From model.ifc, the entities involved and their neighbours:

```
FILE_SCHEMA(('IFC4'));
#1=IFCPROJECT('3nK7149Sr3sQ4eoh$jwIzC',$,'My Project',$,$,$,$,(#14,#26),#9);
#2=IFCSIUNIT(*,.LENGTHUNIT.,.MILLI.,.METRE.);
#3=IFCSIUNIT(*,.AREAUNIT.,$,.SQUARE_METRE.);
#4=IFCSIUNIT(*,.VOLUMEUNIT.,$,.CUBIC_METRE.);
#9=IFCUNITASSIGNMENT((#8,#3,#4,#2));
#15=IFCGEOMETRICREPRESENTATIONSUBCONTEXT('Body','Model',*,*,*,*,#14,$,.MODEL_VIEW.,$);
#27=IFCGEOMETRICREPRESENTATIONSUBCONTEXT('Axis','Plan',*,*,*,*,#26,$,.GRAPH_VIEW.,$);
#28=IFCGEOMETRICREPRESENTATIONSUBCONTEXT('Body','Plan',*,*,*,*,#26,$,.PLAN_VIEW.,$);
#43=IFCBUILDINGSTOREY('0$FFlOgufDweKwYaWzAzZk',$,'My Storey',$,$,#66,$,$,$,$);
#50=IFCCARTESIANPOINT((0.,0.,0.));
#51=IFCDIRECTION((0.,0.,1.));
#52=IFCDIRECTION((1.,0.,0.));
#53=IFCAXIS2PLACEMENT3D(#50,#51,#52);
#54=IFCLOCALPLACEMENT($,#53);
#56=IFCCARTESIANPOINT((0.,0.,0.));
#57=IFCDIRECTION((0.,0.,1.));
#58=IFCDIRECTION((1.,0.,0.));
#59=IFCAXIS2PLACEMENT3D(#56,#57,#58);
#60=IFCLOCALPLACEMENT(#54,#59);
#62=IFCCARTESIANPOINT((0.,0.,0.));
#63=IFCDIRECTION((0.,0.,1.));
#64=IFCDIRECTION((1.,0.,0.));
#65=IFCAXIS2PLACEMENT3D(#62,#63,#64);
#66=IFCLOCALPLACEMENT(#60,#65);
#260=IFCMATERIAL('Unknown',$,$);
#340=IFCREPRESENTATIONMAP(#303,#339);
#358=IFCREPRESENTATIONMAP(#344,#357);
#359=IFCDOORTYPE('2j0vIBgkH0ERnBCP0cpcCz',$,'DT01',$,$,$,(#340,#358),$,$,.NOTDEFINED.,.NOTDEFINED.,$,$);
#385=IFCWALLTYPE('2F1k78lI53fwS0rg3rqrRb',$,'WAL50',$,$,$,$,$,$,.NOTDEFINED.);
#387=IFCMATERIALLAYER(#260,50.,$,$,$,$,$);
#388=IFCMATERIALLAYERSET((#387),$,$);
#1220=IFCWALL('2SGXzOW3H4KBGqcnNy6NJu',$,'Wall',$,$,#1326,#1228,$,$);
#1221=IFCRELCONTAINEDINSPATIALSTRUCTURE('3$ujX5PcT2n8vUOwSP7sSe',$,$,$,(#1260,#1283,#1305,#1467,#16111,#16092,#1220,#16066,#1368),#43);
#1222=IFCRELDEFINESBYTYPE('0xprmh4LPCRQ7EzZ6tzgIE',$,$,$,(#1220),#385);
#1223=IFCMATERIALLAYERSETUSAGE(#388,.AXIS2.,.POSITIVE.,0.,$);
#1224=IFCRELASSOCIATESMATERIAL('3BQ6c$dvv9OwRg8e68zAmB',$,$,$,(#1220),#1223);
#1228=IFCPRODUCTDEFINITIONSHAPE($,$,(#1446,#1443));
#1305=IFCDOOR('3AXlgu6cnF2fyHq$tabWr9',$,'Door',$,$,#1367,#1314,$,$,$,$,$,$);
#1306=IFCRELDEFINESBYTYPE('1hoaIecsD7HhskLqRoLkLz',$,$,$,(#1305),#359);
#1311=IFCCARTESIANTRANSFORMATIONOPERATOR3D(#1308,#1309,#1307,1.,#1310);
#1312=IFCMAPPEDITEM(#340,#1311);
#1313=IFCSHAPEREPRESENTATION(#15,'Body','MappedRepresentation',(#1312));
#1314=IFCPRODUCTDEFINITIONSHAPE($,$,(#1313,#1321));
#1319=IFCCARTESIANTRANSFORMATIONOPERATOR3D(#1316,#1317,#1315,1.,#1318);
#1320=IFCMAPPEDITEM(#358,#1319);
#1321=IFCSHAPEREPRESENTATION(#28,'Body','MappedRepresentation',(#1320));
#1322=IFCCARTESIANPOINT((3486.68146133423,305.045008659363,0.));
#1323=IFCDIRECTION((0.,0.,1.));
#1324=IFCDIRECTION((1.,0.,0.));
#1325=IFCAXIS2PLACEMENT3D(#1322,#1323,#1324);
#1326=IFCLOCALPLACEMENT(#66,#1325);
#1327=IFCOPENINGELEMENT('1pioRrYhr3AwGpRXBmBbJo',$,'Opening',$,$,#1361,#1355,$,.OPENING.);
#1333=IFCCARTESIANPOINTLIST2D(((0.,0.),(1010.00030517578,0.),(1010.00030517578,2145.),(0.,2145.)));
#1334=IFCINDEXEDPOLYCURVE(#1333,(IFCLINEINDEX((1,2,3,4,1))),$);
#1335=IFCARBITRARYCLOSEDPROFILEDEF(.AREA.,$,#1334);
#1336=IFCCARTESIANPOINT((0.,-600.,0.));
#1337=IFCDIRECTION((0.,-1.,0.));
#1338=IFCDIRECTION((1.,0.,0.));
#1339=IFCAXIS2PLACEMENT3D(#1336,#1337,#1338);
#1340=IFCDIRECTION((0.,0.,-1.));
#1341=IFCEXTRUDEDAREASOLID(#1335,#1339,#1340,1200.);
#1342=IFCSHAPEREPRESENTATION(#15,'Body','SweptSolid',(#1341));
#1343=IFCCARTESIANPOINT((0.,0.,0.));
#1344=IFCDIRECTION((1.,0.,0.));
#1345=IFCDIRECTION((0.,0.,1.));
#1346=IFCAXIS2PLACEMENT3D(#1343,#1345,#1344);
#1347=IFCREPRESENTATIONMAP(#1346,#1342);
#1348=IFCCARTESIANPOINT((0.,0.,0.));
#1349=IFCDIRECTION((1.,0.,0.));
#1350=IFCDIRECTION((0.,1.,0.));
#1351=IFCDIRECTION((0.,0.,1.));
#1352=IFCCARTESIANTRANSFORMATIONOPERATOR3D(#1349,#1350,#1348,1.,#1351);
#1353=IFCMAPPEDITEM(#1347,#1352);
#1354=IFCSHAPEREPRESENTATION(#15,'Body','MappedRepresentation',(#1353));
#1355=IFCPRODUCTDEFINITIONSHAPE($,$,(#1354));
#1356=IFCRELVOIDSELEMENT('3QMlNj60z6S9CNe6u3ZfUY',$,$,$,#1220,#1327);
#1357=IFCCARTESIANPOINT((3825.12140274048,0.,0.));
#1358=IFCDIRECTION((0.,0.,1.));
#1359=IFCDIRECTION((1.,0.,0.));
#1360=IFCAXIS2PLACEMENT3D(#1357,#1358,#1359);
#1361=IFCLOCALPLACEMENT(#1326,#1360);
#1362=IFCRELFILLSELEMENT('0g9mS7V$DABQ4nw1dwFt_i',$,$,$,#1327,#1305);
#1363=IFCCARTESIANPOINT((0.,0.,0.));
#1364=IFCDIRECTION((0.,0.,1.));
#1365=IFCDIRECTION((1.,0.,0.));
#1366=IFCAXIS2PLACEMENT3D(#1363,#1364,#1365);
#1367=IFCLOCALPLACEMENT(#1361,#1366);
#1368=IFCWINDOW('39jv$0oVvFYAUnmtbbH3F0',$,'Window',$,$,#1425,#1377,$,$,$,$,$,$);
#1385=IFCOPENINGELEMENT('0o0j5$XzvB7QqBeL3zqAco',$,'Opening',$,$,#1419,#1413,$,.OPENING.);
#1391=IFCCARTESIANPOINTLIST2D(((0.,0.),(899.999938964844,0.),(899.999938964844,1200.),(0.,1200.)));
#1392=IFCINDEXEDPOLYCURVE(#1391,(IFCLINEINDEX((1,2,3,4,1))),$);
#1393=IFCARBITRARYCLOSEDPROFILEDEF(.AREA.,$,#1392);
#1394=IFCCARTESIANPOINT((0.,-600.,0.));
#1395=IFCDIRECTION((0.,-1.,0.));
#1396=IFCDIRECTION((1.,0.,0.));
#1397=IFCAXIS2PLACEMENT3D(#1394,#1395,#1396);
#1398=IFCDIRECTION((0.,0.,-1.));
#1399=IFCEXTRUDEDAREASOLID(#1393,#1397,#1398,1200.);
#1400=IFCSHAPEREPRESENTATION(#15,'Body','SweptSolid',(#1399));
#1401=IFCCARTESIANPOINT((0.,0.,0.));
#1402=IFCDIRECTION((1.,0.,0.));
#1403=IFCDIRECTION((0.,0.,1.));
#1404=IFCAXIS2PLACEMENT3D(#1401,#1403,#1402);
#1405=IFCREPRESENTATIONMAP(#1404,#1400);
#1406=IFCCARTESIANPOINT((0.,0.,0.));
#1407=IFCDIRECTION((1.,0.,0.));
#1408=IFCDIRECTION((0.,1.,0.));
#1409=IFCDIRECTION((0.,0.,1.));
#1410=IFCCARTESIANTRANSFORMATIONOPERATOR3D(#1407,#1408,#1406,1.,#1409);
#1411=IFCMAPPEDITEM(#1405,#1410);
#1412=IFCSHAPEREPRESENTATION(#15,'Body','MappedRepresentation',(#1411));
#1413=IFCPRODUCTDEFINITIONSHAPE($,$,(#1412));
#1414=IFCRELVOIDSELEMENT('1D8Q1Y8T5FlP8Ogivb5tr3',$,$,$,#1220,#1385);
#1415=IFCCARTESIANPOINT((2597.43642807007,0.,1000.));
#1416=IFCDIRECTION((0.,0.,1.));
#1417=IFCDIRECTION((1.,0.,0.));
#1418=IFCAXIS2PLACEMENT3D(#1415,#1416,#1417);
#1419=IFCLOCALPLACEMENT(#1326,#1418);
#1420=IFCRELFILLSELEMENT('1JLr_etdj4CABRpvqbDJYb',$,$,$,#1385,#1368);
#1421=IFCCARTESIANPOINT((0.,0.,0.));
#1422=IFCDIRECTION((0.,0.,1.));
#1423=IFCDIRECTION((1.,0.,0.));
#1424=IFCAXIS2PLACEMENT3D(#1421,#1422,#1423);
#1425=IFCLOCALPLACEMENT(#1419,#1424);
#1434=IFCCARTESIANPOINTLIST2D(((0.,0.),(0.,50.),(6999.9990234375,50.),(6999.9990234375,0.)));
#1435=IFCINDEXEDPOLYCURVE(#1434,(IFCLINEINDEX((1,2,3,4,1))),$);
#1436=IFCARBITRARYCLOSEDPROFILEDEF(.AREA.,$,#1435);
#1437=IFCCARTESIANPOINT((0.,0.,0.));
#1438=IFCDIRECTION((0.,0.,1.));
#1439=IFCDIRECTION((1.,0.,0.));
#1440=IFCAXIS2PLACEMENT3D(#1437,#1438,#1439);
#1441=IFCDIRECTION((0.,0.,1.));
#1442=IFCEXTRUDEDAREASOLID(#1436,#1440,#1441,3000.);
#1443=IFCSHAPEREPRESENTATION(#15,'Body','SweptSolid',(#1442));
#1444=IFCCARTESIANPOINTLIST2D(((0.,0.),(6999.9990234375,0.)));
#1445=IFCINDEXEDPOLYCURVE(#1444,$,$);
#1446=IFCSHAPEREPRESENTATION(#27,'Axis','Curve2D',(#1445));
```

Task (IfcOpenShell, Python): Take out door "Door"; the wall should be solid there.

```python
import ifcopenshell
import ifcopenshell.api.feature
import ifcopenshell.api.root
import ifcopenshell.geom
import ifcopenshell.util.shape

model = ifcopenshell.open("model.ifc")
settings = ifcopenshell.geom.settings()


def volume(element):
    """Net volume in cubic metres, openings subtracted."""
    shape = ifcopenshell.geom.create_shape(settings, element)
    return ifcopenshell.util.shape.get_volume(shape.geometry)


door = model.by_guid("3AXlgu6cnF2fyHq$tabWr9")
opening = door.FillsVoids[0].RelatingOpeningElement
wall = opening.VoidsElements[0].RelatingBuildingElement
before = volume(wall)

ifcopenshell.api.root.remove_product(model, product=door)
ifcopenshell.api.feature.remove_feature(model, feature=opening)

after = volume(wall)

print(f"wall volume {before:.3f} -> {after:.3f} m3")

model.write("model_edited.ifc")
```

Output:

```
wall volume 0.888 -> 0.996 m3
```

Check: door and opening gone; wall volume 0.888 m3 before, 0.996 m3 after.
